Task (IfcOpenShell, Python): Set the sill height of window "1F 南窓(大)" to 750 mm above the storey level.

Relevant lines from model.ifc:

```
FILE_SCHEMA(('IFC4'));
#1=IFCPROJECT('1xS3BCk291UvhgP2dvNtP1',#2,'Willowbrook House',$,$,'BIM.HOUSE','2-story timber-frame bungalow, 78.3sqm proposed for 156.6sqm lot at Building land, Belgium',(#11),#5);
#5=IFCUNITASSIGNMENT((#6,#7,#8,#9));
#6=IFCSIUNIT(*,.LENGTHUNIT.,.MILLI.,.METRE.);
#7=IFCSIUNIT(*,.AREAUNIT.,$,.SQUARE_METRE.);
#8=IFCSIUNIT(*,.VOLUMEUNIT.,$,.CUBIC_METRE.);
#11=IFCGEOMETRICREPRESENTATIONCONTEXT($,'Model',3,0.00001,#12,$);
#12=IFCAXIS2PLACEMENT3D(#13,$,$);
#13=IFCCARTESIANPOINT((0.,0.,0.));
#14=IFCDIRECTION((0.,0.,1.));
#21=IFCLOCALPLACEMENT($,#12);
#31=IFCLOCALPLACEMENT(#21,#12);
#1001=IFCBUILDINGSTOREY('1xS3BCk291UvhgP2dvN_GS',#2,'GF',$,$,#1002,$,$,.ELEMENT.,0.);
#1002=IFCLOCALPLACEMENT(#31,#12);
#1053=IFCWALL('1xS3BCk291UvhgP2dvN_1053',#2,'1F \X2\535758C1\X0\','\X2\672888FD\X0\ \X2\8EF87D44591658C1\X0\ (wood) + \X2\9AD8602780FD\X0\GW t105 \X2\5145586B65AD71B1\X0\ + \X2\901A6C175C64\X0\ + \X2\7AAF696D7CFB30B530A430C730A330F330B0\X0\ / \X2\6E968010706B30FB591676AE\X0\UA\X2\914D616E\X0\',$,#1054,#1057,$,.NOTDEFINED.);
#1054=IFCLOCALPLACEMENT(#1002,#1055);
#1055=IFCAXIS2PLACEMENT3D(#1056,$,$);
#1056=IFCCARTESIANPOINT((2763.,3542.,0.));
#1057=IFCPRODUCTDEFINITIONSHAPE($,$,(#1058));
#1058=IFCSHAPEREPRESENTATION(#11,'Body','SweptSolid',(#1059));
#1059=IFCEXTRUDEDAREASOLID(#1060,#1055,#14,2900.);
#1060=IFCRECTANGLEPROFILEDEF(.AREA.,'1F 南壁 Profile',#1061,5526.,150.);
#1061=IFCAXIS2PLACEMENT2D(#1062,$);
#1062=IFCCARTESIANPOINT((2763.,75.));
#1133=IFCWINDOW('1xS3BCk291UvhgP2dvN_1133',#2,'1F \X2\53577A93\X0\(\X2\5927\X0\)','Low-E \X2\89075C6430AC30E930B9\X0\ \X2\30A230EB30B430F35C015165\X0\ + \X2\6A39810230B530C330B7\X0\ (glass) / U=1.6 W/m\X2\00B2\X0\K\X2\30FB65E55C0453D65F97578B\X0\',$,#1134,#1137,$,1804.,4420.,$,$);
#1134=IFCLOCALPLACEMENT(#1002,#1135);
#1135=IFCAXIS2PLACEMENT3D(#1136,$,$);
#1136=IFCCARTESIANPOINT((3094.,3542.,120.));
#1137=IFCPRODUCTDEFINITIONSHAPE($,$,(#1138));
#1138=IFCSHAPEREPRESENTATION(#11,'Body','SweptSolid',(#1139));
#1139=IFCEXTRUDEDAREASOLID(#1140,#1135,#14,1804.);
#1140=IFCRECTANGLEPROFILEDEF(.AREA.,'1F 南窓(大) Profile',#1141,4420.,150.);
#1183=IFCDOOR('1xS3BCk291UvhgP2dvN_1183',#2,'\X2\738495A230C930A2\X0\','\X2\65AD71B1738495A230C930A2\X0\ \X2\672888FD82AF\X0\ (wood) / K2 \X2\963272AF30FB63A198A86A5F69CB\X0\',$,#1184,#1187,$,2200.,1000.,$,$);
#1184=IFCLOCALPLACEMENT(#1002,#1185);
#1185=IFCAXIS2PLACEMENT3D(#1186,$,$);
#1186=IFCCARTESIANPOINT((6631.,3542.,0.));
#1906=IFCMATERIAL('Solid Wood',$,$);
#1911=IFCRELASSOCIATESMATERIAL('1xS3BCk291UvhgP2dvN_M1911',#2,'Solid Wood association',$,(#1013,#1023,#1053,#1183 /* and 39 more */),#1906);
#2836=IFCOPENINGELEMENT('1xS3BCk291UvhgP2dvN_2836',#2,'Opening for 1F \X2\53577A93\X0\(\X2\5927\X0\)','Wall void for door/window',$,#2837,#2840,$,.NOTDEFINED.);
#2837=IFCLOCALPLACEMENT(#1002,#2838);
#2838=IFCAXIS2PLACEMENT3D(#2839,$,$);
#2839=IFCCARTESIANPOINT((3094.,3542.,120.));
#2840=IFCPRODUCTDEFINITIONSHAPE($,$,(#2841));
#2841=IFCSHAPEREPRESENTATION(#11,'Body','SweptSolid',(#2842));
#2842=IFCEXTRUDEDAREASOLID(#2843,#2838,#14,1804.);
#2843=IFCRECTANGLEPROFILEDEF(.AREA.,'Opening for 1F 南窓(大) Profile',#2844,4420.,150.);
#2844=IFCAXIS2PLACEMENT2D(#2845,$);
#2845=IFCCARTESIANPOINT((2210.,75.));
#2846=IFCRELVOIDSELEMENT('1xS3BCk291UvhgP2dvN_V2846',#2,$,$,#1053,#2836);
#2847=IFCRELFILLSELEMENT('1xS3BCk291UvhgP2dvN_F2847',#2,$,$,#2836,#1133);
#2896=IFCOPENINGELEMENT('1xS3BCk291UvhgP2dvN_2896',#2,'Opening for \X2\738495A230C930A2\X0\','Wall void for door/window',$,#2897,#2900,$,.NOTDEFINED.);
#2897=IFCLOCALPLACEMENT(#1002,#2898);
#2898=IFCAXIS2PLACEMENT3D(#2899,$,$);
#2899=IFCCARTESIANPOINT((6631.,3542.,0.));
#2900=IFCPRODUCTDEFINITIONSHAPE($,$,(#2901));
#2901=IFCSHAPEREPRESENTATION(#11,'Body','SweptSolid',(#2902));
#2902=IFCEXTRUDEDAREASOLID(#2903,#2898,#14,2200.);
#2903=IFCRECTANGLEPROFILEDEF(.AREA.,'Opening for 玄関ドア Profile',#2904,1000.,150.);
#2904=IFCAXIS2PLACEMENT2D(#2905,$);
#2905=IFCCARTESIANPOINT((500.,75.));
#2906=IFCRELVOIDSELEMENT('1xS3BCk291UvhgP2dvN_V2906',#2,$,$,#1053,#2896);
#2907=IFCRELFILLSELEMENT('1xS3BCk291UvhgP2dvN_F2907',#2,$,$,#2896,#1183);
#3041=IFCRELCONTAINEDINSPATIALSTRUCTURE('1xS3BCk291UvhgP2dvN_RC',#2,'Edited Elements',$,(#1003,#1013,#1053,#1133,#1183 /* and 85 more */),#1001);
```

```python
import numpy as np
import ifcopenshell
import ifcopenshell.api.geometry
import ifcopenshell.geom
import ifcopenshell.util.element
import ifcopenshell.util.placement
import ifcopenshell.util.shape
import ifcopenshell.util.unit

model = ifcopenshell.open("model.ifc")
unit_scale = ifcopenshell.util.unit.calculate_unit_scale(model)

window = model.by_guid("1xS3BCk291UvhgP2dvN_1133")
opening = window.FillsVoids[0].RelatingOpeningElement
storey = ifcopenshell.util.element.get_container(window, ifc_class="IfcBuildingStorey")
level = ifcopenshell.util.placement.get_local_placement(storey.ObjectPlacement)[2, 3]

# The opening's origin need not be at the sill, so measure its lowest point.
shape = ifcopenshell.geom.create_shape(ifcopenshell.geom.settings(), opening)
bottom = ifcopenshell.util.shape.get_shape_bottom_elevation(shape, shape.geometry) / unit_scale
dz = level + 750.0 - bottom

shift = np.array([0.0, 0.0, dz])
# The window is not placed relative to its opening, so move both.
for product in (opening, window):
    matrix = ifcopenshell.util.placement.get_local_placement(product.ObjectPlacement)
    matrix[:3, 3] += shift
    ifcopenshell.api.geometry.edit_object_placement(model, product=product, matrix=matrix, is_si=False)

print(f"moved by {dz * unit_scale:+.3f} m")

model.write("model-out.ifc")
```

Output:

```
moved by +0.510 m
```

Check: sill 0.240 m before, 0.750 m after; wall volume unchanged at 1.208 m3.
